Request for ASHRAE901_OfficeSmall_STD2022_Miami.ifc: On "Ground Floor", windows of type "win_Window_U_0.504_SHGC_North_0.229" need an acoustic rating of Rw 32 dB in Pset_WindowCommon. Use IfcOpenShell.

First a look at what the model holds.

```python
import ifcopenshell
import ifcopenshell.util.element

model = ifcopenshell.open("ASHRAE901_OfficeSmall_STD2022_Miami.ifc")
print(model.schema)
storey = next(s for s in model.by_type("IfcBuildingStorey") if s.Name == "Ground Floor")
windows = [e for e in ifcopenshell.util.element.get_decomposition(storey) if e.is_a("IfcWindow")]
seen = {}
for e in windows:
    element_type = ifcopenshell.util.element.get_type(e)
    key = (element_type.Name if element_type != e and element_type else None, ifcopenshell.util.element.get_pset(e, "Pset_WindowCommon", "AcousticRating"))
    seen[key] = seen.get(key, 0) + 1
for (name, value), count in sorted(seen.items(), key=str):
    print(count, "x", name, "|", value)
```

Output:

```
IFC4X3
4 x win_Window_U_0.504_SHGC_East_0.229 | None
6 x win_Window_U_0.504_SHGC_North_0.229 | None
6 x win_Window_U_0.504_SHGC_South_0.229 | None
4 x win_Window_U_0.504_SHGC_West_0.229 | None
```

```python
import ifcopenshell
import ifcopenshell.api.pset
import ifcopenshell.util.element

model = ifcopenshell.open("ASHRAE901_OfficeSmall_STD2022_Miami.ifc")

storey = next(s for s in model.by_type("IfcBuildingStorey") if s.Name == "Ground Floor")
windows = [e for e in ifcopenshell.util.element.get_decomposition(storey) if e.is_a("IfcWindow")]

count = 0
for e in windows:
    element_type = ifcopenshell.util.element.get_type(e)
    if element_type in (None, e) or element_type.Name != "win_Window_U_0.504_SHGC_North_0.229":
        continue
    # add_pset returns the element's existing set when there is one.
    pset = ifcopenshell.api.pset.add_pset(model, product=e, name="Pset_WindowCommon")
    ifcopenshell.api.pset.edit_pset(model, pset=pset, properties={"AcousticRating": "Rw 32 dB"})
    count += 1

print(count, "windows updated")

model.write("ASHRAE901_OfficeSmall_STD2022_Miami-out.ifc")
```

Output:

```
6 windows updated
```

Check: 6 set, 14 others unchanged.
